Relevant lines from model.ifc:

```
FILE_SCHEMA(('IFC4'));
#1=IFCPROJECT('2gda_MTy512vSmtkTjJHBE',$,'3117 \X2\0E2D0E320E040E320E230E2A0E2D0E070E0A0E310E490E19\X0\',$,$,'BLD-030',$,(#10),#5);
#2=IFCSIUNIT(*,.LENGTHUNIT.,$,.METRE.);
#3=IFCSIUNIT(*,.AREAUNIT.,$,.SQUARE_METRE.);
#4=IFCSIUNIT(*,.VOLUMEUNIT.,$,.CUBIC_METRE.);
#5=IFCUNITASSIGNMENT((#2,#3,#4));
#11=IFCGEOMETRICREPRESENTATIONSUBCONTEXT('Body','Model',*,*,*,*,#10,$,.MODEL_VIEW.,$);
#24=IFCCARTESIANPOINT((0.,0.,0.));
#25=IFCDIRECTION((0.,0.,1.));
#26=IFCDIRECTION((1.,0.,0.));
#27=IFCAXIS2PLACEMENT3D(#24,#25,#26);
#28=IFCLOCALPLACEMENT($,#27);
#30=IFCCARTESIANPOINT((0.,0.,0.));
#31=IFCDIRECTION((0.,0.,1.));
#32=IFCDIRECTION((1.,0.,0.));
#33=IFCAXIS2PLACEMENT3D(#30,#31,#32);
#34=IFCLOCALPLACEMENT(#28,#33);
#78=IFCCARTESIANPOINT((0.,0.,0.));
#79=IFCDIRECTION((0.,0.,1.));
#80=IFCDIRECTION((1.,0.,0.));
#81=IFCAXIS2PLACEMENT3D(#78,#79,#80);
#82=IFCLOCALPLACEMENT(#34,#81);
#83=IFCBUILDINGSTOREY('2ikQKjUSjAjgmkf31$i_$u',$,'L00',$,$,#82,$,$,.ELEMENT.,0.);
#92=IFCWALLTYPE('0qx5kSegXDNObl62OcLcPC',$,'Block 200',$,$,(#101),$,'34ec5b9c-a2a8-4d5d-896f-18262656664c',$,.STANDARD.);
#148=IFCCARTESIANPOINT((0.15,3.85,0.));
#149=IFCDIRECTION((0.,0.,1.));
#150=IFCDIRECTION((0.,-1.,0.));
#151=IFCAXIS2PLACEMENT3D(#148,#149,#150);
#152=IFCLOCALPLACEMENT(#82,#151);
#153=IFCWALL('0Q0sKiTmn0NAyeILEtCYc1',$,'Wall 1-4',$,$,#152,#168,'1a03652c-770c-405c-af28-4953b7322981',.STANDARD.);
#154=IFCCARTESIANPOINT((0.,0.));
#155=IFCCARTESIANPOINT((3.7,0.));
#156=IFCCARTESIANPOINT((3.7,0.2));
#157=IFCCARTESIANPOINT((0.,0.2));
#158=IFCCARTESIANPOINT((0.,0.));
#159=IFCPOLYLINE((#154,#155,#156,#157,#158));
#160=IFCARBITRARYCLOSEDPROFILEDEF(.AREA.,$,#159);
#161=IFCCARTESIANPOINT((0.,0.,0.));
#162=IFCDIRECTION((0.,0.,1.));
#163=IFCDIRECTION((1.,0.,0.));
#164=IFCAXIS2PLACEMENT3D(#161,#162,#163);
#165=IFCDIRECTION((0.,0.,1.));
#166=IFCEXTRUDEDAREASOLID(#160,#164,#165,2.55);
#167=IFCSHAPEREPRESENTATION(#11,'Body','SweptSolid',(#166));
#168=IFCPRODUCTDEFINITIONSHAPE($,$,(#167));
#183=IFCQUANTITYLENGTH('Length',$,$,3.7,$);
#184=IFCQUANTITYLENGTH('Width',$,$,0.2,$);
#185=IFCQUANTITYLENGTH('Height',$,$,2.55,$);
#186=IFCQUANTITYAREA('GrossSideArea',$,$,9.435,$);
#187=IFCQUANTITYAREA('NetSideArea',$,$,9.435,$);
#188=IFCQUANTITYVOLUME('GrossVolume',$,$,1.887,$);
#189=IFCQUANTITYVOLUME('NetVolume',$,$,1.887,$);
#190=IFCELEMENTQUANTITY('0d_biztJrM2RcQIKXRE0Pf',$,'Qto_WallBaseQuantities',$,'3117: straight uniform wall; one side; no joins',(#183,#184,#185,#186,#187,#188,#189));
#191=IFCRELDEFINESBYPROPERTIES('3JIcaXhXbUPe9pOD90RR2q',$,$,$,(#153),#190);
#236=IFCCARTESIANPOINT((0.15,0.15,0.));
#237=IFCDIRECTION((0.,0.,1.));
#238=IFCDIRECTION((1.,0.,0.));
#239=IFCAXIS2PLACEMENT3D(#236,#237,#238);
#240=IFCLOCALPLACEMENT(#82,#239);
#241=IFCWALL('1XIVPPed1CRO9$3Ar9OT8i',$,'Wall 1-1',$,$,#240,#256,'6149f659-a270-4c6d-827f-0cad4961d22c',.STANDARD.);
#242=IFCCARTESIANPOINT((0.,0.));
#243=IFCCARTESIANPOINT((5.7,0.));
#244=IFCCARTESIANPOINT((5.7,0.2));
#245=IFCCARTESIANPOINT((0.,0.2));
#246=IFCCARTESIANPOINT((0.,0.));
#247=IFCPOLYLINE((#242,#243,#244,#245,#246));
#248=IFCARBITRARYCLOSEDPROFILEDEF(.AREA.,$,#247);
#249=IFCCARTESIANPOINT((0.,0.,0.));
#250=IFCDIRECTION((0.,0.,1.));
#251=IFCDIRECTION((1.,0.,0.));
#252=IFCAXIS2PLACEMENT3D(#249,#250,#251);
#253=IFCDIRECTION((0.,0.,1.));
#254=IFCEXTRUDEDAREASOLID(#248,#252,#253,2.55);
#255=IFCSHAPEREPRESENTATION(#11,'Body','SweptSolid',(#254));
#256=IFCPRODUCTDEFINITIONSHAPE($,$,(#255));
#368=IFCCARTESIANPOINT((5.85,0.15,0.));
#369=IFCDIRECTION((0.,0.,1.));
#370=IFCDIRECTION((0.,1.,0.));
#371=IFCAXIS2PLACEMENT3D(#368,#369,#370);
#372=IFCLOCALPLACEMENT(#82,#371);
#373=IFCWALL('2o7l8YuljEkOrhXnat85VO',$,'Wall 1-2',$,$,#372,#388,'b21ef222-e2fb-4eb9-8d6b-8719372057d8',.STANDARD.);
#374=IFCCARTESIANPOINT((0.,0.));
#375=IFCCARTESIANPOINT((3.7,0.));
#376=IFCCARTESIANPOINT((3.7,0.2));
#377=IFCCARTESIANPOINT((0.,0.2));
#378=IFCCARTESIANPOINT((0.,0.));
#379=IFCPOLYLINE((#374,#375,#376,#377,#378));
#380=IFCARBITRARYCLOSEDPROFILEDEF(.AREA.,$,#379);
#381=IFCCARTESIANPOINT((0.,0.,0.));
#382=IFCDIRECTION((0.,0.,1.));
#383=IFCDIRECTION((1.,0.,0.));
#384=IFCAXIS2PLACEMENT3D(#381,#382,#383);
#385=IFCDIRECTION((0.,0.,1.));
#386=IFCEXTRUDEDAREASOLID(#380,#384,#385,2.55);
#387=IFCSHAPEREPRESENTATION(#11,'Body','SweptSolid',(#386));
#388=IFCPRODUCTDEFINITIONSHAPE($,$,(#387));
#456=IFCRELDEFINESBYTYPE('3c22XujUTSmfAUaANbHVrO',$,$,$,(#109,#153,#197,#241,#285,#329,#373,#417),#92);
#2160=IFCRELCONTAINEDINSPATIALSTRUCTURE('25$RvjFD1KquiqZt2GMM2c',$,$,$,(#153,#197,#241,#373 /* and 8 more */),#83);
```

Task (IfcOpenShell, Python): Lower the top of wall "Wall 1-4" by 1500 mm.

```python
import ifcopenshell
import ifcopenshell.api.pset
import ifcopenshell.geom
import ifcopenshell.util.element
import ifcopenshell.util.representation
import ifcopenshell.util.shape
import ifcopenshell.util.unit

model = ifcopenshell.open("model.ifc")
unit_scale = ifcopenshell.util.unit.calculate_unit_scale(model)
area_scale = ifcopenshell.util.unit.calculate_unit_scale(model, "AREAUNIT")
volume_scale = ifcopenshell.util.unit.calculate_unit_scale(model, "VOLUMEUNIT")
settings = ifcopenshell.geom.settings()


def volume(element):
    """Net volume in cubic metres, openings subtracted."""
    shape = ifcopenshell.geom.create_shape(settings, element)
    return ifcopenshell.util.shape.get_volume(shape.geometry)


wall = model.by_id(153)
before = volume(wall)

body = ifcopenshell.util.representation.get_representation(wall, "Model", "Body")
solid = body.Items[0]
old_height = solid.Depth
solid.Depth -= 1.5
after = volume(wall)
thickness = 0.2  # wall thickness in metres

# Update the stored height, areas and volumes.
qto = model.by_id(ifcopenshell.util.element.get_pset(wall, "Qto_WallBaseQuantities", should_inherit=False)["id"])
ifcopenshell.api.pset.edit_qto(model, qto=qto, properties={
    "Height": solid.Depth,
    "GrossSideArea": ifcopenshell.util.element.get_pset(wall, "Qto_WallBaseQuantities", "GrossSideArea") * solid.Depth / old_height,
    "NetSideArea": after / thickness / area_scale,
    "GrossVolume": ifcopenshell.util.element.get_pset(wall, "Qto_WallBaseQuantities", "GrossVolume") * solid.Depth / old_height,
    "NetVolume": after / volume_scale,
})

print(f"height {old_height:g} -> {solid.Depth:g}, volume {before:.3f} -> {after:.3f} m3")

model.write("model_rev.ifc")
```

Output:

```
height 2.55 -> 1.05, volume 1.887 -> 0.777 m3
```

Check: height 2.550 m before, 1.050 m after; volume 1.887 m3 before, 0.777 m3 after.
